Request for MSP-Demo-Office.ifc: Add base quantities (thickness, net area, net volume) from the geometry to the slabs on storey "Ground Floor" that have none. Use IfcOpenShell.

First a look at what the model holds.

```python
import ifcopenshell
import ifcopenshell.util.element
import ifcopenshell.util.unit

model = ifcopenshell.open("MSP-Demo-Office.ifc")
print(model.schema)
for unit_type in ("LENGTHUNIT", "AREAUNIT", "VOLUMEUNIT"):
    print(unit_type, ifcopenshell.util.unit.calculate_unit_scale(model, unit_type))
storey = next(s for s in model.by_type("IfcBuildingStorey") if s.Name == "Ground Floor")
slabs = [e for e in ifcopenshell.util.element.get_decomposition(storey) if e.is_a("IfcSlab")]
for e in sorted(slabs, key=lambda e: e.id()):
    print(e.id(), e.is_a(), e.Name, list(ifcopenshell.util.element.get_psets(e, qtos_only=True)), sep=" | ")
```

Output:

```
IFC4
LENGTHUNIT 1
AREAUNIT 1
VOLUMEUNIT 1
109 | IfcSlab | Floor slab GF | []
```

```python
import ifcopenshell
import ifcopenshell.api.pset
import ifcopenshell.geom
import ifcopenshell.util.element
import ifcopenshell.util.shape
import ifcopenshell.util.unit

model = ifcopenshell.open("MSP-Demo-Office.ifc")
unit_scale = ifcopenshell.util.unit.calculate_unit_scale(model)
area_scale = ifcopenshell.util.unit.calculate_unit_scale(model, "AREAUNIT")
volume_scale = ifcopenshell.util.unit.calculate_unit_scale(model, "VOLUMEUNIT")
settings = ifcopenshell.geom.settings()

storey = next(s for s in model.by_type("IfcBuildingStorey") if s.Name == "Ground Floor")
slabs = [e for e in ifcopenshell.util.element.get_decomposition(storey) if e.is_a("IfcSlab")]

for e in sorted(slabs, key=lambda e: e.id()):
    if ifcopenshell.util.element.get_psets(e, qtos_only=True, should_inherit=False):
        continue
    # Geometry comes back in metres, in the element's own axes.
    shape = ifcopenshell.geom.create_shape(settings, e)
    values = {
        "Width": ifcopenshell.util.shape.get_z(shape.geometry) / unit_scale,
        "NetArea": ifcopenshell.util.shape.get_footprint_area(shape.geometry) / area_scale,
        "NetVolume": ifcopenshell.util.shape.get_volume(shape.geometry) / volume_scale,
    }
    qto = ifcopenshell.api.pset.add_qto(model, product=e, name="Qto_SlabBaseQuantities")
    ifcopenshell.api.pset.edit_qto(model, qto=qto, properties=values)
    print(e.id(), {k: round(v, 3) for k, v in values.items()})

model.write("MSP-Demo-Office_updated.ifc")
```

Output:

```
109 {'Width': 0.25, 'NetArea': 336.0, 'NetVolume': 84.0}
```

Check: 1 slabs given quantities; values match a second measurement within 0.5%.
